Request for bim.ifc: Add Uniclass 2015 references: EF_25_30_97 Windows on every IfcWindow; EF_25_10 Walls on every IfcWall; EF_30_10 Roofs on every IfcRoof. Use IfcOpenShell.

First a look at what the model holds.

```python
import ifcopenshell

model = ifcopenshell.open("bim.ifc")
print(model.schema)
print("classifications:", [c.Name for c in model.by_type("IfcClassification")])
for ifc_class in ("IfcDoor", "IfcRoof", "IfcStair", "IfcWall", "IfcWindow"):
    print(ifc_class, len(model.by_type(ifc_class)))
```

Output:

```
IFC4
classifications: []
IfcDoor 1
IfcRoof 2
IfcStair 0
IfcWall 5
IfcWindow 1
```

```python
import ifcopenshell
import ifcopenshell.api.classification

model = ifcopenshell.open("bim.ifc")

system = ifcopenshell.api.classification.add_classification(model, classification="Uniclass 2015")

codes = {
    "IfcWindow": ("EF_25_30_97", "Windows"),
    "IfcWall": ("EF_25_10", "Walls"),
    "IfcRoof": ("EF_30_10", "Roofs"),
}
for ifc_class, (code, name) in codes.items():
    products = model.by_type(ifc_class)
    ifcopenshell.api.classification.add_reference(
        model, products=products, classification=system, identification=code, name=name
    )
    print(code, len(products))

model.write("bim_rev.ifc")
```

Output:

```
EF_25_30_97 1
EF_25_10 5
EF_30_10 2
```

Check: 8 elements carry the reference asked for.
